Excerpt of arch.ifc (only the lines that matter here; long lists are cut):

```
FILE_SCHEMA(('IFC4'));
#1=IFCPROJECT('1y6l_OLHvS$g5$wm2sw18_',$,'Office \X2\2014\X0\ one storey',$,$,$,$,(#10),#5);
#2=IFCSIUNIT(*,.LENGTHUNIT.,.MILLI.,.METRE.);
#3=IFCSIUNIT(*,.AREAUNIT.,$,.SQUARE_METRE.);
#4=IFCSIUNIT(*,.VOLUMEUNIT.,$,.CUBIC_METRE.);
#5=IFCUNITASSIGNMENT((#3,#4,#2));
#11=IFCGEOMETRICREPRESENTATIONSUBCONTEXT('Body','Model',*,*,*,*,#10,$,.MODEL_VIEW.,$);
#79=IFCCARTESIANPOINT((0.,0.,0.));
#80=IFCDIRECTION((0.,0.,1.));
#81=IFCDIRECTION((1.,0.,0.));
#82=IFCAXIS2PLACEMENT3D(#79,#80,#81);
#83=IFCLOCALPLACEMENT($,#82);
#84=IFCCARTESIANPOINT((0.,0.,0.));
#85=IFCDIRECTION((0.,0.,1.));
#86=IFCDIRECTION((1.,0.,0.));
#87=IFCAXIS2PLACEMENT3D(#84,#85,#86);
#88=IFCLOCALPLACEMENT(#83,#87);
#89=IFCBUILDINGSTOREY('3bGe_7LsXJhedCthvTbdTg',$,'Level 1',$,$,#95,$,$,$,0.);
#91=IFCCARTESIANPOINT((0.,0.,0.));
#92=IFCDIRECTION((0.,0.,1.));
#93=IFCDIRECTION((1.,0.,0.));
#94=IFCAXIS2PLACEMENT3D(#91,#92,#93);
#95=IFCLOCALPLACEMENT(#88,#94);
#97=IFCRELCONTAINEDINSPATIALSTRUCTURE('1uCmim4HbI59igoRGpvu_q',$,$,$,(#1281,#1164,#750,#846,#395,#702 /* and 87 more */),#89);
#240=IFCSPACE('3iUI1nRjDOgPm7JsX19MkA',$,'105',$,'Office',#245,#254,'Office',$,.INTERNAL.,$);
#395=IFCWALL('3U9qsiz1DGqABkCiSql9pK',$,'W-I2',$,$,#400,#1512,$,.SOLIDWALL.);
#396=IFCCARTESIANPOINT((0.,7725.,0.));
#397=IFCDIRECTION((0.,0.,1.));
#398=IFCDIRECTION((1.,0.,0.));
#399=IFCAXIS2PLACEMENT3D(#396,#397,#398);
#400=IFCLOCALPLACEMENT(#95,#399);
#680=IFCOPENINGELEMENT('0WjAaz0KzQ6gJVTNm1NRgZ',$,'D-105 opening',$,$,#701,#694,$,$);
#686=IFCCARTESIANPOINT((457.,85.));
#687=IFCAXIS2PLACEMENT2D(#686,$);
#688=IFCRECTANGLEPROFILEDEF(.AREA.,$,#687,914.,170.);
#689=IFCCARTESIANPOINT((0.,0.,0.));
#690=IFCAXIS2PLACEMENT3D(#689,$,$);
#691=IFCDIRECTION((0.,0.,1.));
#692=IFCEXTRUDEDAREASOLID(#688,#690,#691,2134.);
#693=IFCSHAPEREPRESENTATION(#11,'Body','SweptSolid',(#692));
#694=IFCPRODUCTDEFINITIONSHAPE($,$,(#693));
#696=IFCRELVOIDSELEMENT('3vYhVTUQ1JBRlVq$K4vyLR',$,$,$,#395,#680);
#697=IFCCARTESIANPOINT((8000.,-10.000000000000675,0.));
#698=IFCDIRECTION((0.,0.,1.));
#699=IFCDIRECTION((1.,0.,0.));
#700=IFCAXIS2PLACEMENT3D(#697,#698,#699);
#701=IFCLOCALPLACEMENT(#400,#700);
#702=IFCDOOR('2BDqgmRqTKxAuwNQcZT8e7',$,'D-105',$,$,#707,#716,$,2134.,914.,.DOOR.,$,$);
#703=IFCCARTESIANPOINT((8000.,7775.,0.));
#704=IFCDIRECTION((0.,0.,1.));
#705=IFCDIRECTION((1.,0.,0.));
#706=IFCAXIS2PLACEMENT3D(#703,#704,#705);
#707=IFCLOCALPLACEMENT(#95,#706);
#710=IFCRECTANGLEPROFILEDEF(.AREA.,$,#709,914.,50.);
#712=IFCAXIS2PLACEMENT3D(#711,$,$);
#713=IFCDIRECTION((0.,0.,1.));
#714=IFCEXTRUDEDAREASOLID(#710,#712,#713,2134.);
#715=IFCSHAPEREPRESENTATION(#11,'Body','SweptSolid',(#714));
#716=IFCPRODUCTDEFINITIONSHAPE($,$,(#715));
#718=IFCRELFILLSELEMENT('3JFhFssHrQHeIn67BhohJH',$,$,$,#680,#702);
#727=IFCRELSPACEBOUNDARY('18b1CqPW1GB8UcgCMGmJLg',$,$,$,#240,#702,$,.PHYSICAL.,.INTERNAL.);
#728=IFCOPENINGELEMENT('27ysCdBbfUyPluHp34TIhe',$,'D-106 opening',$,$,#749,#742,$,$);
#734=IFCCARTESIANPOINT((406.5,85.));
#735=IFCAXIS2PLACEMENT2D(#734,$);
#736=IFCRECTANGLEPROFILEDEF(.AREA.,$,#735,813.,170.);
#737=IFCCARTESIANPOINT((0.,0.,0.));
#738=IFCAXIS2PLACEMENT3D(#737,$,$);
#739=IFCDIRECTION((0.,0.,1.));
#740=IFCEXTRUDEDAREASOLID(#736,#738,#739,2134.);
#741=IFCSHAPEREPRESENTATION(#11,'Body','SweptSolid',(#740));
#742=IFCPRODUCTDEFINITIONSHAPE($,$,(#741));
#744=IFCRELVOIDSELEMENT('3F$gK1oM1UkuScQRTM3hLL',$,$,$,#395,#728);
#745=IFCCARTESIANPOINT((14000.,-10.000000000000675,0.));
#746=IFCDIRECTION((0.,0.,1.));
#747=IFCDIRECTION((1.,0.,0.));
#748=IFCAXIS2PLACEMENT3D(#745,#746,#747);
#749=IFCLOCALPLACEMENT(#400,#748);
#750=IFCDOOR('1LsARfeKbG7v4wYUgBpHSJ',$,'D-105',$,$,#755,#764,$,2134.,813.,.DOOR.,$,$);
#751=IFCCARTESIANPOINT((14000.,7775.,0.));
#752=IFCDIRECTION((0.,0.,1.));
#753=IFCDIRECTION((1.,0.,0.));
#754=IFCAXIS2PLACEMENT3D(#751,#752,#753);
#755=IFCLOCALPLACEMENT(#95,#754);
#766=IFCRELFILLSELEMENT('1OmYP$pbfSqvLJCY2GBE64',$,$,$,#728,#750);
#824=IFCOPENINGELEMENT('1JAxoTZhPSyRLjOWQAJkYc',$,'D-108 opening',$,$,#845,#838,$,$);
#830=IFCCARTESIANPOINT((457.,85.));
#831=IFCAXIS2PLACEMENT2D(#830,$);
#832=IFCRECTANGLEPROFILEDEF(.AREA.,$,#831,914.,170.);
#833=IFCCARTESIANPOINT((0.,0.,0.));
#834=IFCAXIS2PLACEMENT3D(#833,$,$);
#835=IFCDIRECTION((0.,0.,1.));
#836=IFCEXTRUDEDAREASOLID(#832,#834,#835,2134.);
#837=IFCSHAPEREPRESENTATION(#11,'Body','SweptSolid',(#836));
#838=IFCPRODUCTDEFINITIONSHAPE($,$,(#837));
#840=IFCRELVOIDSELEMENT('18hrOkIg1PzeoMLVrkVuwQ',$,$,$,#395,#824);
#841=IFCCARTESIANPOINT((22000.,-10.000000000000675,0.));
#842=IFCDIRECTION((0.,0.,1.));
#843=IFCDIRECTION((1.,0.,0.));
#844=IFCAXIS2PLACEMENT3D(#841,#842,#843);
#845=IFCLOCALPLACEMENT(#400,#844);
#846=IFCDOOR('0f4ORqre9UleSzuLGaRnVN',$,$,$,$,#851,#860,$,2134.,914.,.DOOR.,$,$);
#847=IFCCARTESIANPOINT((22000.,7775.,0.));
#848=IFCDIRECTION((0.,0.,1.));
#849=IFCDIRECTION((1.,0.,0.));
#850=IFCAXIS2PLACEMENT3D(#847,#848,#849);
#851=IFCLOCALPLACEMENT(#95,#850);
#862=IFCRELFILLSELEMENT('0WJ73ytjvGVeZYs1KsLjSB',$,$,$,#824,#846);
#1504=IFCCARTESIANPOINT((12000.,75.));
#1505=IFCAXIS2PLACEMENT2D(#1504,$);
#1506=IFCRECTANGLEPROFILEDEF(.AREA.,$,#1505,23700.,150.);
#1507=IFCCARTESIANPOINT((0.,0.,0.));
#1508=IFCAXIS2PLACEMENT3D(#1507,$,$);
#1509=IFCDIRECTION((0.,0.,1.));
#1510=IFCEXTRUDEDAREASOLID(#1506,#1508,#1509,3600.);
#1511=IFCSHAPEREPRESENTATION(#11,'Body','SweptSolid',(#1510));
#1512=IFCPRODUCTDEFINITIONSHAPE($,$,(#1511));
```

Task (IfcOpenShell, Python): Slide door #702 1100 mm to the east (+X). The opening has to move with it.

```python
import ifcopenshell
import ifcopenshell.api.geometry
import ifcopenshell.util.placement
import ifcopenshell.util.unit

model = ifcopenshell.open("arch.ifc")
unit_scale = ifcopenshell.util.unit.calculate_unit_scale(model)

door = model.by_id(702)
opening = door.FillsVoids[0].RelatingOpeningElement
wall = opening.VoidsElements[0].RelatingBuildingElement

wall_matrix = ifcopenshell.util.placement.get_local_placement(wall.ObjectPlacement)
shift = wall_matrix[:3, 0] * 1.1 / unit_scale
before = ifcopenshell.util.placement.get_local_placement(door.ObjectPlacement)[:3, 3].copy()

# The door is not placed relative to its opening, so move both.
for product in (opening, door):
    matrix = ifcopenshell.util.placement.get_local_placement(product.ObjectPlacement)
    matrix[:3, 3] += shift
    ifcopenshell.api.geometry.edit_object_placement(model, product=product, matrix=matrix, is_si=False)

after = ifcopenshell.util.placement.get_local_placement(door.ObjectPlacement)[:3, 3]
print("door moved by", (after - before).round(3) + 0.0)

model.write("arch_v2.ifc")
```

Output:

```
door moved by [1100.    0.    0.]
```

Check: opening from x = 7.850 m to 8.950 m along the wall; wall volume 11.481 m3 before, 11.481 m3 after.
